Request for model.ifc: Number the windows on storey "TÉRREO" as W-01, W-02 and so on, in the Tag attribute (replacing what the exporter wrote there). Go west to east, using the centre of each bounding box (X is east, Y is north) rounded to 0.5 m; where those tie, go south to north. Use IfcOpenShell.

First a look at what the model holds.

```python
import ifcopenshell
import ifcopenshell.util.element
import ifcopenshell.util.placement

model = ifcopenshell.open("model.ifc")
print(model.schema)
storey = next(s for s in model.by_type("IfcBuildingStorey") if s.Name == "TÉRREO")
windows = [e for e in ifcopenshell.util.element.get_decomposition(storey) if e.is_a("IfcWindow")]
for e in sorted(windows, key=lambda e: e.id()):
    origin = ifcopenshell.util.placement.get_local_placement(e.ObjectPlacement)[:3, 3]
    print(e.id(), e.Tag, e.Name, origin.round(2) + 0.0, sep=" | ")
```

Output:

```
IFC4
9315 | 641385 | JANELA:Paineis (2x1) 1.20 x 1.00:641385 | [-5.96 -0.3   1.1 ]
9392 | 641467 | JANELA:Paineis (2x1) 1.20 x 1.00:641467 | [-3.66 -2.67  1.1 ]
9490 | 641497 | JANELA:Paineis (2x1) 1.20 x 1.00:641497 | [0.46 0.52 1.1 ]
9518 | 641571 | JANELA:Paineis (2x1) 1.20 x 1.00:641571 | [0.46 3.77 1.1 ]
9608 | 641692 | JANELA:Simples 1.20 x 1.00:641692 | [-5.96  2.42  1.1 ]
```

```python
import ifcopenshell
import ifcopenshell.geom
import ifcopenshell.util.element
import ifcopenshell.util.shape

model = ifcopenshell.open("model.ifc")
settings = ifcopenshell.geom.settings()
settings.set("use-world-coords", True)


def centre(element):
    shape = ifcopenshell.geom.create_shape(settings, element)
    return ifcopenshell.util.shape.get_bbox_centroid(shape.geometry)


storey = next(s for s in model.by_type("IfcBuildingStorey") if s.Name == "TÉRREO")
windows = [e for e in ifcopenshell.util.element.get_decomposition(storey) if e.is_a("IfcWindow")]

# Insertion points can sit at a corner or the storey origin, so sort by the geometry (in metres).
centres = {e: centre(e) for e in windows}
windows.sort(key=lambda e: (round(centres[e][0] / 0.5), centres[e][1]))

for i, e in enumerate(windows, start=1):
    number = f"W-{i:02d}"
    e.Tag = number
    print(e.id(), number)

model.write("model_edited.ifc")
```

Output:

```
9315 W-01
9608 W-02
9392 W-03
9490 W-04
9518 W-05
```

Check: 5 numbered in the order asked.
